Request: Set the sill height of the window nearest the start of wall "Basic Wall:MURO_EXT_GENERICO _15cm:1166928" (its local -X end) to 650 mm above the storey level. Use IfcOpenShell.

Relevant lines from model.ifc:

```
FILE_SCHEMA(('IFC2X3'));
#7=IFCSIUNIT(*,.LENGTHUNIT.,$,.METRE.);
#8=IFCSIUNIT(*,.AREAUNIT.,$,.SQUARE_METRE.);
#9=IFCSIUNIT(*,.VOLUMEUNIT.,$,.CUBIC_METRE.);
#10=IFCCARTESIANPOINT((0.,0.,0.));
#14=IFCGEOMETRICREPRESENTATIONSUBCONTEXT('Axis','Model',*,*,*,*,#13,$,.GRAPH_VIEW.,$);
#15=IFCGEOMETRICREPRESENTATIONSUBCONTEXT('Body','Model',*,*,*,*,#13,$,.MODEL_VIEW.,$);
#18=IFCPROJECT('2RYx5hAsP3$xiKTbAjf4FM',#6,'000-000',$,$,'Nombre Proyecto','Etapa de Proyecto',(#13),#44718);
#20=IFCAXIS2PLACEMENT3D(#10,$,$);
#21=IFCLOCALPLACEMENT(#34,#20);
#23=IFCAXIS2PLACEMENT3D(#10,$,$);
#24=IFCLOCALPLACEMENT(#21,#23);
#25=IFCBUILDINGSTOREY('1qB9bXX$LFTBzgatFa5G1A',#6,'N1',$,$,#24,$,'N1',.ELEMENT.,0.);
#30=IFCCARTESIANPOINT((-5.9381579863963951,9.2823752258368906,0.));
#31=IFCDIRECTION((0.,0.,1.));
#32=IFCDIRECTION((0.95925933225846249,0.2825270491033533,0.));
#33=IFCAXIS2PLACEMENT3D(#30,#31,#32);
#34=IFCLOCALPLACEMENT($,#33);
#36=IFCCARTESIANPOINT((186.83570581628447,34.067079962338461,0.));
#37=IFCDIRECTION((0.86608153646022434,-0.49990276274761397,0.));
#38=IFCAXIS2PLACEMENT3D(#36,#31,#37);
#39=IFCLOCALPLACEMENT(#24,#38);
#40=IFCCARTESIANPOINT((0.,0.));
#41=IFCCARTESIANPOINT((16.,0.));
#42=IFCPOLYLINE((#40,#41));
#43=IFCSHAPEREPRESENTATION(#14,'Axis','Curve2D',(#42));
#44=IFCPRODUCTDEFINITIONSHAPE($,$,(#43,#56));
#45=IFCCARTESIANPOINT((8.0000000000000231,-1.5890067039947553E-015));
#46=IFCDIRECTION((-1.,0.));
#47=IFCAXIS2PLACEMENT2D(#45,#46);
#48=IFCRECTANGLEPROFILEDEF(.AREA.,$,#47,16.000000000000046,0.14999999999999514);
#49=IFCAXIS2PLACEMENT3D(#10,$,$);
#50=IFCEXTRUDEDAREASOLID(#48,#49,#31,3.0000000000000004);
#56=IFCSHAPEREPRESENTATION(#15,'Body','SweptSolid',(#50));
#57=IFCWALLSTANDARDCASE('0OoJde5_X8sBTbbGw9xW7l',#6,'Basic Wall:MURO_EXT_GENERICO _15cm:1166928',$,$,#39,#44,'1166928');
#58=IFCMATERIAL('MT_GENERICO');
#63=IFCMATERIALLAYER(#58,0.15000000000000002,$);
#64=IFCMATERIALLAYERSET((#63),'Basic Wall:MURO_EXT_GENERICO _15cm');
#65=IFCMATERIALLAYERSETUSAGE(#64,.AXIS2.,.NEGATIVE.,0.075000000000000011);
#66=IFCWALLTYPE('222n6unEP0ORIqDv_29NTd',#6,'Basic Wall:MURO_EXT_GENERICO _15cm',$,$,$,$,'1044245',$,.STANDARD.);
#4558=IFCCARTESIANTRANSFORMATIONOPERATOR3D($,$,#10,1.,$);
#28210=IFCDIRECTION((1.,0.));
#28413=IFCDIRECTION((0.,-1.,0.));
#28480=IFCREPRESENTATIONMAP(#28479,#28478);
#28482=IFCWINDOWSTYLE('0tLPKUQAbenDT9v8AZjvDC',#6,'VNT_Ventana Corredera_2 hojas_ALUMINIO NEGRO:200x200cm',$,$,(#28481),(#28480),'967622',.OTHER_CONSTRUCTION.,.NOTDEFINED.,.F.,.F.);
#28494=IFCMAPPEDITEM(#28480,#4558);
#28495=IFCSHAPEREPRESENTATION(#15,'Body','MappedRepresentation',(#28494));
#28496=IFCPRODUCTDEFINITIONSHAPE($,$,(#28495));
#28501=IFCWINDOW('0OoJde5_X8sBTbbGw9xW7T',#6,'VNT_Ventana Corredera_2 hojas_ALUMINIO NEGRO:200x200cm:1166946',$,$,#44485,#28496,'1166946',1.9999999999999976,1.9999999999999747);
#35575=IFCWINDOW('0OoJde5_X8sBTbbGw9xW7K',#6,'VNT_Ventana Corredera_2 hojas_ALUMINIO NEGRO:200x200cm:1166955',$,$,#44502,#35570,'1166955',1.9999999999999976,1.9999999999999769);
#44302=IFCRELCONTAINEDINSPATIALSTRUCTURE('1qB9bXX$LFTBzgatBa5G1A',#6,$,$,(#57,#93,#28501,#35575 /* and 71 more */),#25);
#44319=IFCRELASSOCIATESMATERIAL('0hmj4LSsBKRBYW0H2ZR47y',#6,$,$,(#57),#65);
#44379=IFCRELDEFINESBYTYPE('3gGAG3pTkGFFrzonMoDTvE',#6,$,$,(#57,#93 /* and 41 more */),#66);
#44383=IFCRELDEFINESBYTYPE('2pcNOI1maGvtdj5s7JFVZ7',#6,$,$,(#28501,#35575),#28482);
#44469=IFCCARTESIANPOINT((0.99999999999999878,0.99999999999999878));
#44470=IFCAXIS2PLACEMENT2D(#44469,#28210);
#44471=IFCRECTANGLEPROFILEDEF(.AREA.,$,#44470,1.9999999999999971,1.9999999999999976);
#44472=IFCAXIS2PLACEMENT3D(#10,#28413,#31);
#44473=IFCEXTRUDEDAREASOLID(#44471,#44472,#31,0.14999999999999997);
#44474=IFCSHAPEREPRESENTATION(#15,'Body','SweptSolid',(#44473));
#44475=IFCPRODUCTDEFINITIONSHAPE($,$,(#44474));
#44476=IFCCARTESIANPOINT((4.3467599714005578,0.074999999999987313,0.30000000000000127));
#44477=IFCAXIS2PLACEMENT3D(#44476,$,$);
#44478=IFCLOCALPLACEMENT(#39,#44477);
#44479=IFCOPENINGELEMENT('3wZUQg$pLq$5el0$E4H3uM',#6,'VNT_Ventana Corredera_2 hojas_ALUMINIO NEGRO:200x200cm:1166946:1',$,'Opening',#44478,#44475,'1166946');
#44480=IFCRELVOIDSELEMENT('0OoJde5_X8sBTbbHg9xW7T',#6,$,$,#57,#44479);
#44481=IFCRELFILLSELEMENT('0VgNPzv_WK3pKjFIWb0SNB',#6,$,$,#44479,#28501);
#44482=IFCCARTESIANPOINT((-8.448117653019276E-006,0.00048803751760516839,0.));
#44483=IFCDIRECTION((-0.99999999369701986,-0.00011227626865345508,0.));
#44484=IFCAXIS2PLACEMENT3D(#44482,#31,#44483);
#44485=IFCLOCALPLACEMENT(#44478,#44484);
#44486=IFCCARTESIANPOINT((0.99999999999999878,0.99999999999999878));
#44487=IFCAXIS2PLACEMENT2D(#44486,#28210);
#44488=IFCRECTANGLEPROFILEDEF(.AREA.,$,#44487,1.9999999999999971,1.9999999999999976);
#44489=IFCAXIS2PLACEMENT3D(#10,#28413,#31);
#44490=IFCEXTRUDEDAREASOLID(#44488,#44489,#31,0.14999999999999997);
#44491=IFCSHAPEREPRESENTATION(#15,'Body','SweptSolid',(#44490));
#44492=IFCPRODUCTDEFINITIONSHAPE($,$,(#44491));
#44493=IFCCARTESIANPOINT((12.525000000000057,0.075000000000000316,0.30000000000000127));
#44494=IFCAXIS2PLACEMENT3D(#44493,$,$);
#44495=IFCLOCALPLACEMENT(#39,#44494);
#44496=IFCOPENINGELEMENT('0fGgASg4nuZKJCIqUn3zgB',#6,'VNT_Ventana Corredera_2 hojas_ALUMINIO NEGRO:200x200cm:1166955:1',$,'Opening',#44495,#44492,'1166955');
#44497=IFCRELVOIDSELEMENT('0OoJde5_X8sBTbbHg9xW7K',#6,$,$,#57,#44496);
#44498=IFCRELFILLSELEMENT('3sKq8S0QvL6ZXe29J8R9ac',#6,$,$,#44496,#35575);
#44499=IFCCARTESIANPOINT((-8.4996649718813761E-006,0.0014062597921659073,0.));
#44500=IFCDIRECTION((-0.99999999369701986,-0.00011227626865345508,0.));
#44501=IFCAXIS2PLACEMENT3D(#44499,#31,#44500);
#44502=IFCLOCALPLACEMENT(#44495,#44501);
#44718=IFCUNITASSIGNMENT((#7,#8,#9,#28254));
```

```python
import numpy as np
import ifcopenshell
import ifcopenshell.api.geometry
import ifcopenshell.geom
import ifcopenshell.util.element
import ifcopenshell.util.placement
import ifcopenshell.util.shape
import ifcopenshell.util.unit

model = ifcopenshell.open("model.ifc")
unit_scale = ifcopenshell.util.unit.calculate_unit_scale(model)

window = model.by_guid("0OoJde5_X8sBTbbGw9xW7T")
opening = window.FillsVoids[0].RelatingOpeningElement
storey = ifcopenshell.util.element.get_container(window, ifc_class="IfcBuildingStorey")
level = ifcopenshell.util.placement.get_local_placement(storey.ObjectPlacement)[2, 3]

# The opening's origin need not be at the sill, so measure its lowest point.
shape = ifcopenshell.geom.create_shape(ifcopenshell.geom.settings(), opening)
bottom = ifcopenshell.util.shape.get_shape_bottom_elevation(shape, shape.geometry) / unit_scale
dz = level + 0.65 / unit_scale - bottom

shift = np.array([0.0, 0.0, dz])
# The window is placed relative to its opening, so it follows when the opening moves.
matrix = ifcopenshell.util.placement.get_local_placement(opening.ObjectPlacement)
matrix[:3, 3] += shift
ifcopenshell.api.geometry.edit_object_placement(
    model, product=opening, matrix=matrix, is_si=False, should_transform_children=True
)

print(f"moved by {dz * unit_scale:+.3f} m")

model.write("model_updated.ifc")
```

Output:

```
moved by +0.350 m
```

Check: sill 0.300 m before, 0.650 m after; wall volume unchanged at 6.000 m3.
